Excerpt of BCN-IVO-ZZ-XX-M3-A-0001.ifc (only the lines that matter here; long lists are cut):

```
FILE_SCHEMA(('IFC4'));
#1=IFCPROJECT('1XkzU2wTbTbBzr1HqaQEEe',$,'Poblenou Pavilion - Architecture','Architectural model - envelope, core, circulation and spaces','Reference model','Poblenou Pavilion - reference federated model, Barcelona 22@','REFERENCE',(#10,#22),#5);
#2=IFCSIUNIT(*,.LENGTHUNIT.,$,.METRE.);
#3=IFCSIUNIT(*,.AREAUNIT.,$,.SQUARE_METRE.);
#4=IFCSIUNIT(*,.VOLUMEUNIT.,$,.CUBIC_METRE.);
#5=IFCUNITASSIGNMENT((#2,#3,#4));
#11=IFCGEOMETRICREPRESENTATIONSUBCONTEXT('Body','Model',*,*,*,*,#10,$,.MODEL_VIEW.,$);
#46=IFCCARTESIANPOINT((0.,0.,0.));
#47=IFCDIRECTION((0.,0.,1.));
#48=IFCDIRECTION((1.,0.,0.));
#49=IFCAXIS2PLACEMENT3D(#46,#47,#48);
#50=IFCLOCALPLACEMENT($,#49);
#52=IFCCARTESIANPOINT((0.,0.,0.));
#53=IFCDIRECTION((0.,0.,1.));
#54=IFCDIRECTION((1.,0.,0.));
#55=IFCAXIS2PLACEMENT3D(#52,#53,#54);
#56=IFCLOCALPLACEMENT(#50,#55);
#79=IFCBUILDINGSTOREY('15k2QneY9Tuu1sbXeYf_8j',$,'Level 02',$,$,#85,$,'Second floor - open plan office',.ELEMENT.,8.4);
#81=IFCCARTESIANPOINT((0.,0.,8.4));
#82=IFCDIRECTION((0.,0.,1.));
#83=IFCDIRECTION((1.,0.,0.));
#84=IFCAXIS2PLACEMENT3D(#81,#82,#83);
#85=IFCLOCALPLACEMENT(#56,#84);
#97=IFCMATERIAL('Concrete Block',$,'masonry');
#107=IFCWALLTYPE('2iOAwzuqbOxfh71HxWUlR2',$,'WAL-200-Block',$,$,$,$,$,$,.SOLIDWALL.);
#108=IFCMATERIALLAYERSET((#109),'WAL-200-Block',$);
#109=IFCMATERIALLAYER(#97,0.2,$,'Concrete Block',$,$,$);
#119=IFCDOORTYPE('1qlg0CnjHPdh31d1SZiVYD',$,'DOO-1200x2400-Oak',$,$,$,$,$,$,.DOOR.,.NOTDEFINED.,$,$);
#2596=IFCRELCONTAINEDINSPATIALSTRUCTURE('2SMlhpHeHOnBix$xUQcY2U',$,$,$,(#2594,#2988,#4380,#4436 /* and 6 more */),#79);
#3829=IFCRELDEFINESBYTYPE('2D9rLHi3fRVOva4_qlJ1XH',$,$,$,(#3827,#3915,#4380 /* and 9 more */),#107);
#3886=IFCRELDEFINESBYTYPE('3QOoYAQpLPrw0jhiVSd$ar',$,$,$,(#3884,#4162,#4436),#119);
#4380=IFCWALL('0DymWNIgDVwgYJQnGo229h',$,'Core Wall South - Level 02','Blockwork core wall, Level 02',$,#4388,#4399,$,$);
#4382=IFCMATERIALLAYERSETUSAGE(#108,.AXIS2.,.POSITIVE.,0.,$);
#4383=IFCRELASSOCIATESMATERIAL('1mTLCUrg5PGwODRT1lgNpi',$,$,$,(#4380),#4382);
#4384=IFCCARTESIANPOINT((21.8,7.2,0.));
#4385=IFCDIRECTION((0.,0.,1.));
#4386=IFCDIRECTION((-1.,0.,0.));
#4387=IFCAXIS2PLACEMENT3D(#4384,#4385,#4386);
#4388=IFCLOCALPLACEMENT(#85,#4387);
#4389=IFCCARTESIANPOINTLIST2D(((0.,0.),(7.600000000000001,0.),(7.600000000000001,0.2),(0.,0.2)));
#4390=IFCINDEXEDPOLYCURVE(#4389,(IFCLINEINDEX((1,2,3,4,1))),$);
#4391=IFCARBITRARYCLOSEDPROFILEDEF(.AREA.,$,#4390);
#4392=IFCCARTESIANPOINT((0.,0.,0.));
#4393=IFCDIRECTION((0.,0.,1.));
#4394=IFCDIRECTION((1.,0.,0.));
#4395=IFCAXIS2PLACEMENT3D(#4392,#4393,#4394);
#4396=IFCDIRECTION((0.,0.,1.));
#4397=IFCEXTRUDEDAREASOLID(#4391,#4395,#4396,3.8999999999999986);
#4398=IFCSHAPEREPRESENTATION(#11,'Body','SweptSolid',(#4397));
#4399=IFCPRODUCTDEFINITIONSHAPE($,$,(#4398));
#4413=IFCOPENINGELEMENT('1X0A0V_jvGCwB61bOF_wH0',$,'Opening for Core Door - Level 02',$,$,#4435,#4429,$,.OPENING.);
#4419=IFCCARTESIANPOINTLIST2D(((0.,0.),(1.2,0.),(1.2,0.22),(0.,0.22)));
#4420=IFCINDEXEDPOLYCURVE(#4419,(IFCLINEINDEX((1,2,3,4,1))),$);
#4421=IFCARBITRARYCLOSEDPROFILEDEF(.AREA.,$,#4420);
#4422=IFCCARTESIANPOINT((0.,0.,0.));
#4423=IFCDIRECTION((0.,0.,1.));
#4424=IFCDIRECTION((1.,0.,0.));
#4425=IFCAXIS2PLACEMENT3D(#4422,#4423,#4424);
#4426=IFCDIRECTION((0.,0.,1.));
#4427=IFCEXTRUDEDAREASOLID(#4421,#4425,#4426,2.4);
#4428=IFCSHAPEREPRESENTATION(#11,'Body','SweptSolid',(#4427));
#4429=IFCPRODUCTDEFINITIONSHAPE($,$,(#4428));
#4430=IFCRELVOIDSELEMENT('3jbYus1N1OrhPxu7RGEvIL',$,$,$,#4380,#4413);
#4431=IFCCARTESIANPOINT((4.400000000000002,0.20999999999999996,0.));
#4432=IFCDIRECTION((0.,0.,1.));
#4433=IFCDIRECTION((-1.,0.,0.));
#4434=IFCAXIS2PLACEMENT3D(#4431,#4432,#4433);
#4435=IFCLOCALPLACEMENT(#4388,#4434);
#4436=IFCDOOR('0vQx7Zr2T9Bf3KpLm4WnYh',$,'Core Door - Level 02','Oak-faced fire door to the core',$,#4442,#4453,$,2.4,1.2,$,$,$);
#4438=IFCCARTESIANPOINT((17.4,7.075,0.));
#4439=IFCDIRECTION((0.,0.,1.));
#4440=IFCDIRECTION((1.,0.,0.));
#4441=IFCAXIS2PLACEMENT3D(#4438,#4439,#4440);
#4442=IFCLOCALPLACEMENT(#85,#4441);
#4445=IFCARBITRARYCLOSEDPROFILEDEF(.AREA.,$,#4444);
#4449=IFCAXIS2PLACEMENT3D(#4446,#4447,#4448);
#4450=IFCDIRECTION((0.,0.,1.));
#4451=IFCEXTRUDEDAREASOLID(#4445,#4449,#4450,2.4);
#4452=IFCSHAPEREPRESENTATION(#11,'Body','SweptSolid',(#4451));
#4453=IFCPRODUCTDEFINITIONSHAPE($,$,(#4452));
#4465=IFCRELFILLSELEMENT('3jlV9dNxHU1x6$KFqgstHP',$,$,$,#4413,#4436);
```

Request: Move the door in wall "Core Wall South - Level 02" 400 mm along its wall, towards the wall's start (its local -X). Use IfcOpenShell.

```python
import ifcopenshell
import ifcopenshell.api.geometry
import ifcopenshell.util.placement

model = ifcopenshell.open("BCN-IVO-ZZ-XX-M3-A-0001.ifc")

door = model.by_guid("0vQx7Zr2T9Bf3KpLm4WnYh")
opening = door.FillsVoids[0].RelatingOpeningElement
wall = opening.VoidsElements[0].RelatingBuildingElement

wall_matrix = ifcopenshell.util.placement.get_local_placement(wall.ObjectPlacement)
shift = wall_matrix[:3, 0] * -0.4
before = ifcopenshell.util.placement.get_local_placement(door.ObjectPlacement)[:3, 3].copy()

# The door is not placed relative to its opening, so move both.
for product in (opening, door):
    matrix = ifcopenshell.util.placement.get_local_placement(product.ObjectPlacement)
    matrix[:3, 3] += shift
    ifcopenshell.api.geometry.edit_object_placement(model, product=product, matrix=matrix, is_si=False)

after = ifcopenshell.util.placement.get_local_placement(door.ObjectPlacement)[:3, 3]
print("door moved by", (after - before).round(3) + 0.0)

model.write("BCN-IVO-ZZ-XX-M3-A-0001_v2.ifc")
```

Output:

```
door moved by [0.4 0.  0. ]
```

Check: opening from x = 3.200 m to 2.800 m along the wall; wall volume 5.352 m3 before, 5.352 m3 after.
